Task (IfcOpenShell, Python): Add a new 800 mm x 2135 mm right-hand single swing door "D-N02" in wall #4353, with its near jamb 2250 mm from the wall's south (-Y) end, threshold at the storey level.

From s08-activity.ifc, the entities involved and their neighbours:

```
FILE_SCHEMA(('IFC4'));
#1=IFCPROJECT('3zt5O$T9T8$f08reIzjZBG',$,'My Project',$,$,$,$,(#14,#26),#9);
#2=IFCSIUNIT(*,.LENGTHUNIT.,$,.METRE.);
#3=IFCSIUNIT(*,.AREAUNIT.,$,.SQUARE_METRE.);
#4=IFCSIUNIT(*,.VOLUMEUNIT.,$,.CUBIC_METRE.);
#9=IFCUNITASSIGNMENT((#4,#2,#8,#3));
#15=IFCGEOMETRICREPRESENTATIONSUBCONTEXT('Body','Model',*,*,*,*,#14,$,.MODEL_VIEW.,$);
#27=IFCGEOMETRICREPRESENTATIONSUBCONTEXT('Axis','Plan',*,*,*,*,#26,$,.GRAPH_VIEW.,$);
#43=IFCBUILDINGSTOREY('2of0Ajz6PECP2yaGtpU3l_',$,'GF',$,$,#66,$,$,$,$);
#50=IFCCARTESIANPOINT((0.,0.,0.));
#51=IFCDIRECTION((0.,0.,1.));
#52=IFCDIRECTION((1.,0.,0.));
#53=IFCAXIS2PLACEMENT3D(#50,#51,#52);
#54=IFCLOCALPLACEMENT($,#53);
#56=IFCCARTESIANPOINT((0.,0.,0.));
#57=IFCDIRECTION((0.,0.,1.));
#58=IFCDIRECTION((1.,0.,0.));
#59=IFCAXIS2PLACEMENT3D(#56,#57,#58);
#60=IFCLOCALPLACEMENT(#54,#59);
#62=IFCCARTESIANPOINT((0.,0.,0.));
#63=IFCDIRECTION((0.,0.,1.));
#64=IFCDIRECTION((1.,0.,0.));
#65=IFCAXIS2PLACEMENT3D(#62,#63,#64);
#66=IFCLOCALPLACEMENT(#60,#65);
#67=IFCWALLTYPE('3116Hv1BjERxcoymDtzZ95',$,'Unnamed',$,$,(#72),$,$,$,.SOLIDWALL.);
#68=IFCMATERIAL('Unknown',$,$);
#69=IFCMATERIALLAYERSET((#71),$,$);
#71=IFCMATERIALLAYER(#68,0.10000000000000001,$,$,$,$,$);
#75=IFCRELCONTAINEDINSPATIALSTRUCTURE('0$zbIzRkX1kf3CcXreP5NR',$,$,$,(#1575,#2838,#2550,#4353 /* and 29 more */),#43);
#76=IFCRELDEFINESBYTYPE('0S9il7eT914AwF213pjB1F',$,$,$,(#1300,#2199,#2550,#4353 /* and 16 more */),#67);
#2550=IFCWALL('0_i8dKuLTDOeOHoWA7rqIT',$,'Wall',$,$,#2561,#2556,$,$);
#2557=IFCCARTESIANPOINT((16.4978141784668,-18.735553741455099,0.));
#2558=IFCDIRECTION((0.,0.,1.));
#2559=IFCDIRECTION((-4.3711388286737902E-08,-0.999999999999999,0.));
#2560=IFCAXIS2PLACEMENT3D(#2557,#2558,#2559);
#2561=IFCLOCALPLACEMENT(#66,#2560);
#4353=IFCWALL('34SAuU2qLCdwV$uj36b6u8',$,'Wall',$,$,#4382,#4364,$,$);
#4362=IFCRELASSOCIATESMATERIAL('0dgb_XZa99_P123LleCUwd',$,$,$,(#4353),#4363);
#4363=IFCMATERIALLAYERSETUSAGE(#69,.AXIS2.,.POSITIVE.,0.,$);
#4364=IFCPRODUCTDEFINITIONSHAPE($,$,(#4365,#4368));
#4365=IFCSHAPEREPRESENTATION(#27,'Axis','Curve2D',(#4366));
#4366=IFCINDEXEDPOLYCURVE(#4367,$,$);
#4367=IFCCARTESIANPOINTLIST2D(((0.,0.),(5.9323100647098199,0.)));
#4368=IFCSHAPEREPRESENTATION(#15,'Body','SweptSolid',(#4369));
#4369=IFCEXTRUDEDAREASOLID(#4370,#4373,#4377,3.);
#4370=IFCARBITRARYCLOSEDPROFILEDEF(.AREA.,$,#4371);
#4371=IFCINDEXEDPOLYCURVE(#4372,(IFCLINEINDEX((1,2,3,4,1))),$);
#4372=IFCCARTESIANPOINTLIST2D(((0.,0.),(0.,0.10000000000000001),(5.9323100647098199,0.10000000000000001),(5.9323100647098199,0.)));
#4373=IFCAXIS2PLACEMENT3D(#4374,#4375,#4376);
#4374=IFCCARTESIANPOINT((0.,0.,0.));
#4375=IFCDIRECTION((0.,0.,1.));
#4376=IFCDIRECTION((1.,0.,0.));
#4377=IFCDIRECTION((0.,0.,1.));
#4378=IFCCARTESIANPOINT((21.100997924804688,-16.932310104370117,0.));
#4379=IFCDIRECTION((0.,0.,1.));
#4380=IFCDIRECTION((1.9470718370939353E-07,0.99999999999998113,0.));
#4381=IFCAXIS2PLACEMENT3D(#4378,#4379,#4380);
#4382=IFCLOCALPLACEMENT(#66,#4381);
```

```python
import numpy as np
import ifcopenshell
import ifcopenshell.api.feature
import ifcopenshell.api.geometry
import ifcopenshell.api.root
import ifcopenshell.api.spatial
import ifcopenshell.geom
import ifcopenshell.util.element
import ifcopenshell.util.placement
import ifcopenshell.util.representation
import ifcopenshell.util.shape
import ifcopenshell.util.unit

model = ifcopenshell.open("s08-activity.ifc")
unit_scale = ifcopenshell.util.unit.calculate_unit_scale(model)
settings = ifcopenshell.geom.settings()


def volume(element):
    """Net volume in cubic metres, openings subtracted."""
    shape = ifcopenshell.geom.create_shape(settings, element)
    return ifcopenshell.util.shape.get_volume(shape.geometry)


wall = model.by_guid("34SAuU2qLCdwV$uj36b6u8")
storey = ifcopenshell.util.element.get_container(wall, ifc_class="IfcBuildingStorey")
context = ifcopenshell.util.representation.get_context(model, "Model", "Body", "MODEL_VIEW")
before = volume(wall)

width, height, from_end, sill = 0.8, 2.135, 2.25, 0.0  # metres

# The wall runs along its own X axis, and the end named is its -X end.
wall_shape = ifcopenshell.geom.create_shape(settings, wall)
x, y, z = ifcopenshell.util.shape.get_vertices(wall_shape.geometry).T
start = x.min() + from_end
face, thickness = float(y.min()), float(y.max() - y.min())
wall_matrix = ifcopenshell.util.placement.get_local_placement(wall.ObjectPlacement)
level = ifcopenshell.util.placement.get_local_placement(storey.ObjectPlacement)[2, 3]


def in_wall(x, y):
    """Placement at x, y metres in the wall's axes, at sill height."""
    matrix = wall_matrix.copy()
    matrix[:, 3] = wall_matrix @ np.array([x / unit_scale, y / unit_scale, 0.0, 1.0])
    matrix[2, 3] = level + sill / unit_scale
    return matrix


# Opening: a box that overshoots both wall faces by 50 mm.
opening = ifcopenshell.api.root.create_entity(model, ifc_class="IfcOpeningElement", predefined_type="OPENING")
box = ifcopenshell.api.geometry.add_wall_representation(
    model, context=context, length=width, height=height, thickness=thickness + 0.1
)
ifcopenshell.api.geometry.assign_representation(model, product=opening, representation=box)
ifcopenshell.api.geometry.edit_object_placement(model, product=opening, matrix=in_wall(start, face - 0.05), is_si=False)
ifcopenshell.api.feature.add_feature(model, feature=opening, element=wall)

door = ifcopenshell.api.root.create_entity(model, ifc_class="IfcDoor", name="D-N02", predefined_type="DOOR")
door.OverallWidth, door.OverallHeight = width / unit_scale, height / unit_scale
door.OperationType = "SINGLE_SWING_RIGHT"
body = ifcopenshell.api.geometry.add_door_representation(
    model,
    context=context,
    overall_width=door.OverallWidth,
    overall_height=door.OverallHeight,
    operation_type="SINGLE_SWING_RIGHT",
    lining_properties={"LiningDepth": thickness / unit_scale, "ThresholdDepth": thickness / unit_scale},
)
ifcopenshell.api.geometry.assign_representation(model, product=door, representation=body)
ifcopenshell.api.spatial.assign_container(model, products=[door], relating_structure=storey)
ifcopenshell.api.feature.add_filling(model, opening=opening, element=door)

# The lining spans the wall, so the door starts at the wall face.
ifcopenshell.api.geometry.edit_object_placement(model, product=door, matrix=in_wall(start, face), is_si=False)

after = volume(wall)

print(f"wall volume {before:.3f} -> {after:.3f} m3")

model.write("s08-activity_v2.ifc")
```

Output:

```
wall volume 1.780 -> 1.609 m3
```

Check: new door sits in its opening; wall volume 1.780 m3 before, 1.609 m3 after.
